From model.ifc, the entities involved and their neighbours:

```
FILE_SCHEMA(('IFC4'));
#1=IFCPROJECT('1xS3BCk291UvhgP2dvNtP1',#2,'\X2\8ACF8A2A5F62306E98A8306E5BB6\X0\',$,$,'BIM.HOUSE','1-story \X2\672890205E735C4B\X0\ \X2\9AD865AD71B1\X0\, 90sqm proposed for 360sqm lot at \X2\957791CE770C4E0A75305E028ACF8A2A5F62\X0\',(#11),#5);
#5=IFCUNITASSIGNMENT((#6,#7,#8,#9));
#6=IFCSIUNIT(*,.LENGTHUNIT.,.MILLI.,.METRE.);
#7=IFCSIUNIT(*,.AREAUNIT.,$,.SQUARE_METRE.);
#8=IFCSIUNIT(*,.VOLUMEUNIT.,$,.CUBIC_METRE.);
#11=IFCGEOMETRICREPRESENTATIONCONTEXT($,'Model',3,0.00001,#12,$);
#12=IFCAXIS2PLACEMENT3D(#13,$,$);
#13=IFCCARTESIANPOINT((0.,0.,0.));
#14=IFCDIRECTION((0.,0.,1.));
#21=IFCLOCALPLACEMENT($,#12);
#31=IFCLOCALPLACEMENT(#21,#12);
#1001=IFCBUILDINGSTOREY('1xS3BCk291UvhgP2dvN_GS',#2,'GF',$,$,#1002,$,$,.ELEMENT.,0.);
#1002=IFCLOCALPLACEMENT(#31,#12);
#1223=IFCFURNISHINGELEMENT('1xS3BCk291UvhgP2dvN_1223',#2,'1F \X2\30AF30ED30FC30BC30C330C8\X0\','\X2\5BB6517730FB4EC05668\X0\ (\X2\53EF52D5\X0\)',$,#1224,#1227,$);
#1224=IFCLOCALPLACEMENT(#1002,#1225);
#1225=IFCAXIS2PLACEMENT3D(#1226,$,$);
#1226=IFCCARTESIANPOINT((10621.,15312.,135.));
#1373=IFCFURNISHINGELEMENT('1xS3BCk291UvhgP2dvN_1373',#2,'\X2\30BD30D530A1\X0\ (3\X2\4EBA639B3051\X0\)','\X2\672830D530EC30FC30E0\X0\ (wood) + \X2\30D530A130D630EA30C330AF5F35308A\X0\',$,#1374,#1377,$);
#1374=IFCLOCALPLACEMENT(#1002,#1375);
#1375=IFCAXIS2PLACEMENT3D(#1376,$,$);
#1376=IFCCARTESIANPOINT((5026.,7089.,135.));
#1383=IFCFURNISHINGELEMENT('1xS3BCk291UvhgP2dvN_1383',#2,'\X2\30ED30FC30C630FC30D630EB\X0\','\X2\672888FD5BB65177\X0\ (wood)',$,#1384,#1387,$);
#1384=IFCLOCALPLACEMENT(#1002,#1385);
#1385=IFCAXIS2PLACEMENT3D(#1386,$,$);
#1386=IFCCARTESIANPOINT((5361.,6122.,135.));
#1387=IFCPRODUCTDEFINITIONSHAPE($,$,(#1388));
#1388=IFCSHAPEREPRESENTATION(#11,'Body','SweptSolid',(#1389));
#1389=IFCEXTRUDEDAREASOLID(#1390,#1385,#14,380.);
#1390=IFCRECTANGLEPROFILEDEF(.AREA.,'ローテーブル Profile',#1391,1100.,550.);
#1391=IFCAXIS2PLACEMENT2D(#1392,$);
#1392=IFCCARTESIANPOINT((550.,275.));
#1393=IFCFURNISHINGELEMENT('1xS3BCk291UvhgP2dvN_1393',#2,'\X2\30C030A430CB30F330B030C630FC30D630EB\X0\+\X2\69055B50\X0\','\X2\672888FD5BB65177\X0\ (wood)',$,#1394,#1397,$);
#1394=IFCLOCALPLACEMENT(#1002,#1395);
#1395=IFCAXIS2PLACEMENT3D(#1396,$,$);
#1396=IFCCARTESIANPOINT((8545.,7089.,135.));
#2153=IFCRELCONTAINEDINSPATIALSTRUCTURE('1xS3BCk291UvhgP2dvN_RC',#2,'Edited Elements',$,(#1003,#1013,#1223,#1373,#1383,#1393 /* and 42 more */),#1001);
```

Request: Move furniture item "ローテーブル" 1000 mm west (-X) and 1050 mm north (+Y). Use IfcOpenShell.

```python
import ifcopenshell
import ifcopenshell.api.geometry
import ifcopenshell.util.placement
import ifcopenshell.util.unit

model = ifcopenshell.open("model.ifc")
unit_scale = ifcopenshell.util.unit.calculate_unit_scale(model)

item = model.by_id(1383)
matrix = ifcopenshell.util.placement.get_local_placement(item.ObjectPlacement)
matrix[0, 3] -= 1 / unit_scale
matrix[1, 3] += 1.05 / unit_scale
ifcopenshell.api.geometry.edit_object_placement(model, product=item, matrix=matrix, is_si=False)

print(ifcopenshell.util.placement.get_local_placement(item.ObjectPlacement).round(3) + 0.0)

model.write("model_rev.ifc")
```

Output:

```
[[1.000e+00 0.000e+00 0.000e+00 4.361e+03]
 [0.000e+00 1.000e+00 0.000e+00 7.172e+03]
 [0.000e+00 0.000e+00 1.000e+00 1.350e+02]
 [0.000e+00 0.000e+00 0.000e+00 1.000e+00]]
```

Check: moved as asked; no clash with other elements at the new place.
